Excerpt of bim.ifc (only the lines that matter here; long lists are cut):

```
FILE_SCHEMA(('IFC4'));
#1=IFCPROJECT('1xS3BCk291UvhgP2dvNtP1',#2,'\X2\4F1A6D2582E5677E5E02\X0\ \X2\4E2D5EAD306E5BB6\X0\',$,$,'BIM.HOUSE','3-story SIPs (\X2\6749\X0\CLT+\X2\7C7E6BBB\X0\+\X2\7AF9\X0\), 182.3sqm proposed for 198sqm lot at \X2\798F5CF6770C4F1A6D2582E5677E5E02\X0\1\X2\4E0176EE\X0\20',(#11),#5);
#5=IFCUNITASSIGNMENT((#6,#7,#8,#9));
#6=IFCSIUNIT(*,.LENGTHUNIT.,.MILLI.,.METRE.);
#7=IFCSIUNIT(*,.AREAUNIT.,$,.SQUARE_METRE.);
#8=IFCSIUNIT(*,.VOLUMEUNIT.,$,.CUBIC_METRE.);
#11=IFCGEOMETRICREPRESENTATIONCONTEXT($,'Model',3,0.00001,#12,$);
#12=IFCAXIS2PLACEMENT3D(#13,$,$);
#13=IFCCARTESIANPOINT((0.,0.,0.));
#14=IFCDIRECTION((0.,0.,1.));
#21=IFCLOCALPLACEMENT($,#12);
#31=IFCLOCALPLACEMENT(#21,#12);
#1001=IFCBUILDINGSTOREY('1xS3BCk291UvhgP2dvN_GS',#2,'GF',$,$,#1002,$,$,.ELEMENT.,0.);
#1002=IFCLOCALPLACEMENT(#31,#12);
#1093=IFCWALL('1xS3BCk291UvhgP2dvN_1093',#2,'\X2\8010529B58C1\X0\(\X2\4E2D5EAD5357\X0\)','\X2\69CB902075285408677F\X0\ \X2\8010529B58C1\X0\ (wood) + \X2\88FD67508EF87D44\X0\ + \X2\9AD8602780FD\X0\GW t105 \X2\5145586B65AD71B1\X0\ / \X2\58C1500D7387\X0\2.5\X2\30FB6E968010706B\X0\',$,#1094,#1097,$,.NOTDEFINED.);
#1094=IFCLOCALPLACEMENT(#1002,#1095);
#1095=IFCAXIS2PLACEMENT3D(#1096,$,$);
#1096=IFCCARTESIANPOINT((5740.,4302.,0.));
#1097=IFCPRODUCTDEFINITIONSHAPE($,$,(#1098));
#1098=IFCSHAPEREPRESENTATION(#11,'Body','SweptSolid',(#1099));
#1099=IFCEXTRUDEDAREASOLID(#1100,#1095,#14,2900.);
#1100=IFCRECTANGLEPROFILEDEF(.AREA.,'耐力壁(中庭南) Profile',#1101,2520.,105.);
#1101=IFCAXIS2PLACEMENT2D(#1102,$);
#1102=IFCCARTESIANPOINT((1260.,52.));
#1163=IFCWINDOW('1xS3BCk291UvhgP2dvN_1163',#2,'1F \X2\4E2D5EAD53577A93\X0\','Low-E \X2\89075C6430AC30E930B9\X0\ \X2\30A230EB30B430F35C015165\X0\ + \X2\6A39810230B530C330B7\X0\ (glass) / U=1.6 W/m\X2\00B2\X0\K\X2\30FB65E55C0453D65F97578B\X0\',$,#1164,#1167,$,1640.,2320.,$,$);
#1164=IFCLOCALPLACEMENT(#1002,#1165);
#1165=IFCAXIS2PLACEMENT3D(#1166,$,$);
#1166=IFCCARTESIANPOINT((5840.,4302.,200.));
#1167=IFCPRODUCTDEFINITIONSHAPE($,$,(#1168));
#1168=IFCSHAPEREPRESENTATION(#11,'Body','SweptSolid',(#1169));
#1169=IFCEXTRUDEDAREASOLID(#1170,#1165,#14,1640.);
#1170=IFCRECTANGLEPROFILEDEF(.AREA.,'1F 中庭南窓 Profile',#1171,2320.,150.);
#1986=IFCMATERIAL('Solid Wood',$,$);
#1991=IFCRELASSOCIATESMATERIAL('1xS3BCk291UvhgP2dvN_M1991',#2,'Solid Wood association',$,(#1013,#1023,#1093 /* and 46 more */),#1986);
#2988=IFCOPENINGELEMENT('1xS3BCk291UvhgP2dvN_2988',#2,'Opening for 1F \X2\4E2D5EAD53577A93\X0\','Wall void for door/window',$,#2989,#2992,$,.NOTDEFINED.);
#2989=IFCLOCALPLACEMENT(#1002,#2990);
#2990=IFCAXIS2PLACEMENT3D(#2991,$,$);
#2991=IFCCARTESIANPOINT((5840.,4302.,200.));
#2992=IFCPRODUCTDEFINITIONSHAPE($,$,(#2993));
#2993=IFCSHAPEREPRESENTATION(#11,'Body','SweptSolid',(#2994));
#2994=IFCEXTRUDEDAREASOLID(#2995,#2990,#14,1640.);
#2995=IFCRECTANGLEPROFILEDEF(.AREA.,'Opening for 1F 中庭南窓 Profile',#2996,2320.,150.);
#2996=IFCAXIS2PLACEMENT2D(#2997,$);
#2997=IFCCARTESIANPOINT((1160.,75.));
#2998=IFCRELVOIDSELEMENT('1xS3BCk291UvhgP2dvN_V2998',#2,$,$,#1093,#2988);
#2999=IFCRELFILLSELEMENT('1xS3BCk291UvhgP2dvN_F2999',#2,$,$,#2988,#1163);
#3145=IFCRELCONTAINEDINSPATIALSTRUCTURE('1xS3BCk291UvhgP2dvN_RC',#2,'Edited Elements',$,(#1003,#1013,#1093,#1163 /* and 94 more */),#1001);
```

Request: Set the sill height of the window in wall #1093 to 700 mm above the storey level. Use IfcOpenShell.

```python
import numpy as np
import ifcopenshell
import ifcopenshell.api.geometry
import ifcopenshell.geom
import ifcopenshell.util.element
import ifcopenshell.util.placement
import ifcopenshell.util.shape
import ifcopenshell.util.unit

model = ifcopenshell.open("bim.ifc")
unit_scale = ifcopenshell.util.unit.calculate_unit_scale(model)

window = model.by_id(1163)
opening = window.FillsVoids[0].RelatingOpeningElement
storey = ifcopenshell.util.element.get_container(window, ifc_class="IfcBuildingStorey")
level = ifcopenshell.util.placement.get_local_placement(storey.ObjectPlacement)[2, 3]

# The opening's origin need not be at the sill, so measure its lowest point.
shape = ifcopenshell.geom.create_shape(ifcopenshell.geom.settings(), opening)
bottom = ifcopenshell.util.shape.get_shape_bottom_elevation(shape, shape.geometry) / unit_scale
dz = level + 700.0 - bottom

shift = np.array([0.0, 0.0, dz])
# The window is not placed relative to its opening, so move both.
for product in (opening, window):
    matrix = ifcopenshell.util.placement.get_local_placement(product.ObjectPlacement)
    matrix[:3, 3] += shift
    ifcopenshell.api.geometry.edit_object_placement(model, product=product, matrix=matrix, is_si=False)

print(f"moved by {dz * unit_scale:+.3f} m")

model.write("bim_updated.ifc")
```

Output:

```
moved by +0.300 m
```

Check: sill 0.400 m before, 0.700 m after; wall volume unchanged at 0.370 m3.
